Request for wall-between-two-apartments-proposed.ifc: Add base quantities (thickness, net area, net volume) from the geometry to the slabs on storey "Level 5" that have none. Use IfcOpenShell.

First a look at what the model holds.

```python
import ifcopenshell
import ifcopenshell.util.element
import ifcopenshell.util.unit

model = ifcopenshell.open("wall-between-two-apartments-proposed.ifc")
print(model.schema)
for unit_type in ("LENGTHUNIT", "AREAUNIT", "VOLUMEUNIT"):
    print(unit_type, ifcopenshell.util.unit.calculate_unit_scale(model, unit_type))
storey = next(s for s in model.by_type("IfcBuildingStorey") if s.Name == "Level 5")
slabs = [e for e in ifcopenshell.util.element.get_decomposition(storey) if e.is_a("IfcSlab")]
for e in sorted(slabs, key=lambda e: e.id()):
    print(e.id(), e.is_a(), e.Name, list(ifcopenshell.util.element.get_psets(e, qtos_only=True)), sep=" | ")
```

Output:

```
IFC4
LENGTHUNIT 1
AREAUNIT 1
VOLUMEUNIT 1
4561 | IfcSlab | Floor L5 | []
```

```python
import ifcopenshell
import ifcopenshell.api.pset
import ifcopenshell.geom
import ifcopenshell.util.element
import ifcopenshell.util.shape
import ifcopenshell.util.unit

model = ifcopenshell.open("wall-between-two-apartments-proposed.ifc")
unit_scale = ifcopenshell.util.unit.calculate_unit_scale(model)
area_scale = ifcopenshell.util.unit.calculate_unit_scale(model, "AREAUNIT")
volume_scale = ifcopenshell.util.unit.calculate_unit_scale(model, "VOLUMEUNIT")
settings = ifcopenshell.geom.settings()

storey = next(s for s in model.by_type("IfcBuildingStorey") if s.Name == "Level 5")
slabs = [e for e in ifcopenshell.util.element.get_decomposition(storey) if e.is_a("IfcSlab")]

for e in sorted(slabs, key=lambda e: e.id()):
    if ifcopenshell.util.element.get_psets(e, qtos_only=True, should_inherit=False):
        continue
    # Geometry comes back in metres, in the element's own axes.
    shape = ifcopenshell.geom.create_shape(settings, e)
    values = {
        "Width": ifcopenshell.util.shape.get_z(shape.geometry) / unit_scale,
        "NetArea": ifcopenshell.util.shape.get_footprint_area(shape.geometry) / area_scale,
        "NetVolume": ifcopenshell.util.shape.get_volume(shape.geometry) / volume_scale,
    }
    qto = ifcopenshell.api.pset.add_qto(model, product=e, name="Qto_SlabBaseQuantities")
    ifcopenshell.api.pset.edit_qto(model, qto=qto, properties=values)
    print(e.id(), {k: round(v, 3) for k, v in values.items()})

model.write("wall-between-two-apartments-proposed_v2.ifc")
```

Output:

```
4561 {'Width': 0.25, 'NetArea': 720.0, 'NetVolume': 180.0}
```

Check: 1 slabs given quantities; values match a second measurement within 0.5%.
